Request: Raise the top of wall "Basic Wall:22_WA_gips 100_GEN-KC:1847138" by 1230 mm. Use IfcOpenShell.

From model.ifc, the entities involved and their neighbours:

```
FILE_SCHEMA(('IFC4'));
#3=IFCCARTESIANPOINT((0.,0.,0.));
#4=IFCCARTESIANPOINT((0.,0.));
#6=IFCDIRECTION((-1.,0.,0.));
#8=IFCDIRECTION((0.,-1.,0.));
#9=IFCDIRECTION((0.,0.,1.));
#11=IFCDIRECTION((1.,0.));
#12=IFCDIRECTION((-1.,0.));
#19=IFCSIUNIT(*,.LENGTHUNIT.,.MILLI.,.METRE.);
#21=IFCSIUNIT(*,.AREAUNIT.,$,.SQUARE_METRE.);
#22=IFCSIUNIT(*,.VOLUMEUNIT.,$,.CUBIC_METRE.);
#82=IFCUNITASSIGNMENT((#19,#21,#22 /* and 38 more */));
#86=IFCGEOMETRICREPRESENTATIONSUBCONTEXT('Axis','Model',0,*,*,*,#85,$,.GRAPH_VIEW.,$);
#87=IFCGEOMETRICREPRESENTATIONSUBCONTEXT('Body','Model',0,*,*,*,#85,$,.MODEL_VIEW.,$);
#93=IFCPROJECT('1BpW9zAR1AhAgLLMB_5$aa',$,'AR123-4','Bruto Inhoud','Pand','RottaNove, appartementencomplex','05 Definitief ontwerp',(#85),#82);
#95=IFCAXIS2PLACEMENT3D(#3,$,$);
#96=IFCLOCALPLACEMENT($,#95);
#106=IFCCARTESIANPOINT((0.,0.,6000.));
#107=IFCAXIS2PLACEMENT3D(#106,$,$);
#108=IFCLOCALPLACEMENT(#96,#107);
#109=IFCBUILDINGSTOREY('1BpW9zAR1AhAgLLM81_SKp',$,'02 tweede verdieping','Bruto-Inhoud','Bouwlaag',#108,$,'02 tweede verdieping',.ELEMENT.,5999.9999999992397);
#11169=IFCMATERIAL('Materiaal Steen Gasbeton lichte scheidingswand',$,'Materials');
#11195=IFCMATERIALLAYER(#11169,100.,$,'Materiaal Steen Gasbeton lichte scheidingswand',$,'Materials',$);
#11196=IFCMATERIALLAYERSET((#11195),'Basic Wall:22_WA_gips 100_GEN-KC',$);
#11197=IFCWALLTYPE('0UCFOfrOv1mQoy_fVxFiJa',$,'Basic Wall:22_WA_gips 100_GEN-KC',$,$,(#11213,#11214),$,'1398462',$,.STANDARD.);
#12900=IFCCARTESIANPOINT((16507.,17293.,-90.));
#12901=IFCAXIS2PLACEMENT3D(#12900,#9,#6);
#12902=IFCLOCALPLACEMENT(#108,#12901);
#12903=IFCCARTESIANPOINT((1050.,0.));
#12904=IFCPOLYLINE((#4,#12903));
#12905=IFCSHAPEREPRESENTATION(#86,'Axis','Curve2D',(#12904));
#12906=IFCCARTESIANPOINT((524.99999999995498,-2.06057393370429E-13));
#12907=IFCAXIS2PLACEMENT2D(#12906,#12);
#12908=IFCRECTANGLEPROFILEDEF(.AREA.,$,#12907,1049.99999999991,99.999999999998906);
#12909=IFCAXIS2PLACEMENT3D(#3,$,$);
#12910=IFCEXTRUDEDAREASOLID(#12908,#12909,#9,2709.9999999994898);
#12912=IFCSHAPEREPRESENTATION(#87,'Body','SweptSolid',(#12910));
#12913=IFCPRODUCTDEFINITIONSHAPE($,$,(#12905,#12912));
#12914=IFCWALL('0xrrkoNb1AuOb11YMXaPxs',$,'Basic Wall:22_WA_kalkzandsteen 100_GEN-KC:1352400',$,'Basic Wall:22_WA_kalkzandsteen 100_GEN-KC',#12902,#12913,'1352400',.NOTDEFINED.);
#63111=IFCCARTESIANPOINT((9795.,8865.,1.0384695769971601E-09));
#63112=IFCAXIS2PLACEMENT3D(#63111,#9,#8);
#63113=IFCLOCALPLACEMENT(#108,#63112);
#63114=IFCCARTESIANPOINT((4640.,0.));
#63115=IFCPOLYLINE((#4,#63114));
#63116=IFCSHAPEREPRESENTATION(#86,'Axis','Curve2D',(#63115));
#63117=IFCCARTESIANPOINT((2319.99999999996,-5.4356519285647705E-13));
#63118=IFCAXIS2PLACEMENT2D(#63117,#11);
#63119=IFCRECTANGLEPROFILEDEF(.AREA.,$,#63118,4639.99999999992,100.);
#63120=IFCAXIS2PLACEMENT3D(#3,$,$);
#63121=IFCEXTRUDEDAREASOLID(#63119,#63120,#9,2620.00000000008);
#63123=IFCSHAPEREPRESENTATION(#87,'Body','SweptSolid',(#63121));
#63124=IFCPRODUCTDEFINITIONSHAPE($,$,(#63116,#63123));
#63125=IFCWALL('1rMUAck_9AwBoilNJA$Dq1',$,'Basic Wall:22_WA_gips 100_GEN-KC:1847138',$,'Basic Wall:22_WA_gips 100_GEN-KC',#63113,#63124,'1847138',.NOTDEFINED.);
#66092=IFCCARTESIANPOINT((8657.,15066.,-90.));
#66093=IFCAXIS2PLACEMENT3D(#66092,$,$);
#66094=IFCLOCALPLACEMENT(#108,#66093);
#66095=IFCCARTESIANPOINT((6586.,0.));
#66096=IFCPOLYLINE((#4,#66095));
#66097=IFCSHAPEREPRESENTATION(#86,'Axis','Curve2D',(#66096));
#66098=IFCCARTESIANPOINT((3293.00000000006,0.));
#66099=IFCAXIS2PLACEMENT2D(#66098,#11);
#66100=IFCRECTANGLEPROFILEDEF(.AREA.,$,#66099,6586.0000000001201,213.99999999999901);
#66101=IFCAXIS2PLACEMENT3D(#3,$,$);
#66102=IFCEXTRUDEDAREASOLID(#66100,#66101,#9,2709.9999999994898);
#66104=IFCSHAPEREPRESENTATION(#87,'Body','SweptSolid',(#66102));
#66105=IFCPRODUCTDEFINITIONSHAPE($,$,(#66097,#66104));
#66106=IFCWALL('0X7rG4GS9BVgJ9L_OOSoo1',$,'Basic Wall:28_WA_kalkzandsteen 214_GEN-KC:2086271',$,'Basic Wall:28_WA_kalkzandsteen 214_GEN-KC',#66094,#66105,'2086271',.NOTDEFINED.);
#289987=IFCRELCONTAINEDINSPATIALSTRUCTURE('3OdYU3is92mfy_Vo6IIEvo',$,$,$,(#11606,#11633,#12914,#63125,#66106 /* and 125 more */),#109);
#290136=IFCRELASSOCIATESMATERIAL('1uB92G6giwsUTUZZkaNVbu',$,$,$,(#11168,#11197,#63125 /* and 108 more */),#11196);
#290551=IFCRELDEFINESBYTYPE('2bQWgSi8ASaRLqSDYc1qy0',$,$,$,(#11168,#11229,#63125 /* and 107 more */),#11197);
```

```python
import ifcopenshell
import ifcopenshell.geom
import ifcopenshell.util.representation
import ifcopenshell.util.shape

model = ifcopenshell.open("model.ifc")
settings = ifcopenshell.geom.settings()


def volume(element):
    """Net volume in cubic metres, openings subtracted."""
    shape = ifcopenshell.geom.create_shape(settings, element)
    return ifcopenshell.util.shape.get_volume(shape.geometry)


wall = model.by_id(63125)
before = volume(wall)

body = ifcopenshell.util.representation.get_representation(wall, "Model", "Body")
solid = body.Items[0]
old_height = solid.Depth
solid.Depth += 1230.0
after = volume(wall)

print(f"height {old_height:g} -> {solid.Depth:g}, volume {before:.3f} -> {after:.3f} m3")

model.write("model_rev.ifc")
```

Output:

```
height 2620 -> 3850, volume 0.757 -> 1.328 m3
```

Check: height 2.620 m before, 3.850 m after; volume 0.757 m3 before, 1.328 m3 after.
